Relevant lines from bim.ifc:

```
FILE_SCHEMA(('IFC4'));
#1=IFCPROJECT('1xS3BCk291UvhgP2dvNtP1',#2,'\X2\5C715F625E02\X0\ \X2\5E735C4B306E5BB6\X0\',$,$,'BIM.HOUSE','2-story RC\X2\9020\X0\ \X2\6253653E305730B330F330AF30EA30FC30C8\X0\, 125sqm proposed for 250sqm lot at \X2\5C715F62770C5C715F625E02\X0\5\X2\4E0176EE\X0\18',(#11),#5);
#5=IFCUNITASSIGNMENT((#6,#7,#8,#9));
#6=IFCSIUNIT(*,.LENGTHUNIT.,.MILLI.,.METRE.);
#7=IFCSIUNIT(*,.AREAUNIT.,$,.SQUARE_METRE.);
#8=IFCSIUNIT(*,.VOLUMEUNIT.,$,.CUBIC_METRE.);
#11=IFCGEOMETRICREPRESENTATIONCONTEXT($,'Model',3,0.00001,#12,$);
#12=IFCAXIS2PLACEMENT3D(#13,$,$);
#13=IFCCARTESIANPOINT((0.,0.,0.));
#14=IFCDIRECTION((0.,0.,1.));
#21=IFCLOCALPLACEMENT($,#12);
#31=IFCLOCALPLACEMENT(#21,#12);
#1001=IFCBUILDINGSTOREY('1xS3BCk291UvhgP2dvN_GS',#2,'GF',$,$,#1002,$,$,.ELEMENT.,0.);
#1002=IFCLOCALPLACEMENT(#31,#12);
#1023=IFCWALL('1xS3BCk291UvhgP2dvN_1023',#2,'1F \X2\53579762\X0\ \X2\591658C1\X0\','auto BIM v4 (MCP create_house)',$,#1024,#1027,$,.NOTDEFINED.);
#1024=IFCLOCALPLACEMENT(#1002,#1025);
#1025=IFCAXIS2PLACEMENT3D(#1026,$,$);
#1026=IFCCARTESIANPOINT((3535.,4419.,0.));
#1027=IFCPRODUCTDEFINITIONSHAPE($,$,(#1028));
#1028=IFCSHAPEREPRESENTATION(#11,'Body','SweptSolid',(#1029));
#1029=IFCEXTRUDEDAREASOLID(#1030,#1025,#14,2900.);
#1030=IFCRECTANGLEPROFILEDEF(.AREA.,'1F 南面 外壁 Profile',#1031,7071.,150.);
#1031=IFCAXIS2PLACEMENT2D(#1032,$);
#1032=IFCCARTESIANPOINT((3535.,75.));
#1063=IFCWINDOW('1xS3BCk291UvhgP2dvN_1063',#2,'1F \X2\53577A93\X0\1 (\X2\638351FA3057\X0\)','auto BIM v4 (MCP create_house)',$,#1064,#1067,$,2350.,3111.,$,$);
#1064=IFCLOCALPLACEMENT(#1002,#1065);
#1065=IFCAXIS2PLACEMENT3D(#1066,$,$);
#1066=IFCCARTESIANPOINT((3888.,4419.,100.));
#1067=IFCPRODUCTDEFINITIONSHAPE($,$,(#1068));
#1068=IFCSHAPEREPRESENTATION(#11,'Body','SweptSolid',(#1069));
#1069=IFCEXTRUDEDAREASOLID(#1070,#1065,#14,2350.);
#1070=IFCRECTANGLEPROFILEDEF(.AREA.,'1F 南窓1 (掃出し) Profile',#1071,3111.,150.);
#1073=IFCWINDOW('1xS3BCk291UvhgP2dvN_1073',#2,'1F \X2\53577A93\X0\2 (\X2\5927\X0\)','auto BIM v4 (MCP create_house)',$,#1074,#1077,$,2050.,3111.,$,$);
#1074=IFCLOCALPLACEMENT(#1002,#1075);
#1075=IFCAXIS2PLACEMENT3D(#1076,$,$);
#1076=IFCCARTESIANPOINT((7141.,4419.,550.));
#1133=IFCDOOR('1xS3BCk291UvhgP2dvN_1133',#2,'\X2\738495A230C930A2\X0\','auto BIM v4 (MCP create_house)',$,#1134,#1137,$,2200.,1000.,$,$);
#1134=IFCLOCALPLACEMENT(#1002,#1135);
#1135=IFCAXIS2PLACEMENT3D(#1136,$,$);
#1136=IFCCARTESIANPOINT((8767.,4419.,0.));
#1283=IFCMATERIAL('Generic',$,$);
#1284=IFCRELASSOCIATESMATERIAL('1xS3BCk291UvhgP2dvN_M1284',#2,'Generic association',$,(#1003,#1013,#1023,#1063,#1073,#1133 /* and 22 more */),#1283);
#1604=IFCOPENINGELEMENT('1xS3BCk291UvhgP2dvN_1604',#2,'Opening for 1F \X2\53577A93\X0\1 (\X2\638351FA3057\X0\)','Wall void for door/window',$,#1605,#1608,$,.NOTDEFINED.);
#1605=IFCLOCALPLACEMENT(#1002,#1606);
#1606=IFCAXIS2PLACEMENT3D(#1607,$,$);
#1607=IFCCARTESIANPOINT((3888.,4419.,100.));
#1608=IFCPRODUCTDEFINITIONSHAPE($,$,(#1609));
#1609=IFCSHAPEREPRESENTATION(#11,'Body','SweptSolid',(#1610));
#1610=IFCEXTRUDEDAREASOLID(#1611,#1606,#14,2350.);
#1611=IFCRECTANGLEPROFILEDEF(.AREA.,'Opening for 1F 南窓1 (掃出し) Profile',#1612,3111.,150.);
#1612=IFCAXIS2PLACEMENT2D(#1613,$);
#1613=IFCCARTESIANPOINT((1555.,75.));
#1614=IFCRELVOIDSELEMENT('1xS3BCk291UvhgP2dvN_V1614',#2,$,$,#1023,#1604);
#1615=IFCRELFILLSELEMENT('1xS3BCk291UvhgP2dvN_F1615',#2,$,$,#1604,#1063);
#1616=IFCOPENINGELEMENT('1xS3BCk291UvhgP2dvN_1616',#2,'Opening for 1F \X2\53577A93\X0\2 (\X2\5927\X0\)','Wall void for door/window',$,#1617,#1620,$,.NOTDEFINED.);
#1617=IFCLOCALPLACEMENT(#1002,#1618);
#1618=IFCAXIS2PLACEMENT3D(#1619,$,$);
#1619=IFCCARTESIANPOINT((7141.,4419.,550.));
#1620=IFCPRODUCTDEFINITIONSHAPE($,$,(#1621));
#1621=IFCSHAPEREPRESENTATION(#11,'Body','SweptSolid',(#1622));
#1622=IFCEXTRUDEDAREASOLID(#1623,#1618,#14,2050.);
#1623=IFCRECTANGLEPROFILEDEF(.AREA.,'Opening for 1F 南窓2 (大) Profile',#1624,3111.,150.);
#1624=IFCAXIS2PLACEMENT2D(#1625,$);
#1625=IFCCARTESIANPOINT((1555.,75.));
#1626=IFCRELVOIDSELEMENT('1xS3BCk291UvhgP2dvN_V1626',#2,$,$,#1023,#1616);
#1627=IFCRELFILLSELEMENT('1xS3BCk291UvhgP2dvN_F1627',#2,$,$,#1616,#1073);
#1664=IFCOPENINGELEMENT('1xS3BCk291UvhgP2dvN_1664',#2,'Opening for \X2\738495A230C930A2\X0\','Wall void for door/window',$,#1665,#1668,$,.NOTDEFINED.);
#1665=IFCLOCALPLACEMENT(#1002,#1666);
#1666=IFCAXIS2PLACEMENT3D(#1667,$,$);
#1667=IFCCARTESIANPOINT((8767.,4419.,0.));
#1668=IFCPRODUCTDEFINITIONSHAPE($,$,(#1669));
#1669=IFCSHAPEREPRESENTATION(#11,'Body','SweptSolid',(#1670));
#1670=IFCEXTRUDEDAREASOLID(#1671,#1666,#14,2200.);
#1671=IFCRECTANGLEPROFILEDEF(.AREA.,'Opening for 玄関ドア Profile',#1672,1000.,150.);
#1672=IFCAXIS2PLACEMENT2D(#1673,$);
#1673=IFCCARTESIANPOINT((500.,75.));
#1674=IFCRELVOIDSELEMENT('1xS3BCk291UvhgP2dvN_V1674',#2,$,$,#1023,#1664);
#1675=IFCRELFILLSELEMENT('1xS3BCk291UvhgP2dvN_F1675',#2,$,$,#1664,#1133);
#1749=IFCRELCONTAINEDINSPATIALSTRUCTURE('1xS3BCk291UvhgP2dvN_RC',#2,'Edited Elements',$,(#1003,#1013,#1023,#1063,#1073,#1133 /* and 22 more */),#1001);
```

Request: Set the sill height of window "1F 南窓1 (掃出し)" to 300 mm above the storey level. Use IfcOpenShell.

```python
import numpy as np
import ifcopenshell
import ifcopenshell.api.geometry
import ifcopenshell.geom
import ifcopenshell.util.element
import ifcopenshell.util.placement
import ifcopenshell.util.shape
import ifcopenshell.util.unit

model = ifcopenshell.open("bim.ifc")
unit_scale = ifcopenshell.util.unit.calculate_unit_scale(model)

window = model.by_id(1063)
opening = window.FillsVoids[0].RelatingOpeningElement
storey = ifcopenshell.util.element.get_container(window, ifc_class="IfcBuildingStorey")
level = ifcopenshell.util.placement.get_local_placement(storey.ObjectPlacement)[2, 3]

# The opening's origin need not be at the sill, so measure its lowest point.
shape = ifcopenshell.geom.create_shape(ifcopenshell.geom.settings(), opening)
bottom = ifcopenshell.util.shape.get_shape_bottom_elevation(shape, shape.geometry) / unit_scale
dz = level + 0.3 / unit_scale - bottom

shift = np.array([0.0, 0.0, dz])
# The window is not placed relative to its opening, so move both.
for product in (opening, window):
    matrix = ifcopenshell.util.placement.get_local_placement(product.ObjectPlacement)
    matrix[:3, 3] += shift
    ifcopenshell.api.geometry.edit_object_placement(model, product=product, matrix=matrix, is_si=False)

print(f"moved by {dz * unit_scale:+.3f} m")

model.write("bim-out.ifc")
```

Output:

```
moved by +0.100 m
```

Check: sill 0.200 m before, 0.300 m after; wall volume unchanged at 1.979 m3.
